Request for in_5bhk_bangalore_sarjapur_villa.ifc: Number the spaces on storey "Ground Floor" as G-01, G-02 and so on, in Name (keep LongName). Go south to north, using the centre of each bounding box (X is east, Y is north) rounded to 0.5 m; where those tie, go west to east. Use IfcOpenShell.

First a look at what the model holds.

```python
import ifcopenshell
import ifcopenshell.util.element
import ifcopenshell.util.placement

model = ifcopenshell.open("in_5bhk_bangalore_sarjapur_villa.ifc")
print(model.schema)
storey = next(s for s in model.by_type("IfcBuildingStorey") if s.Name == "Ground Floor")
spaces = [e for e in ifcopenshell.util.element.get_decomposition(storey) if e.is_a("IfcSpace")]
for e in sorted(spaces, key=lambda e: e.id()):
    origin = ifcopenshell.util.placement.get_local_placement(e.ObjectPlacement)[:3, 3]
    print(e.id(), e.Name, e.LongName, origin.round(2) + 0.0, sep=" | ")
```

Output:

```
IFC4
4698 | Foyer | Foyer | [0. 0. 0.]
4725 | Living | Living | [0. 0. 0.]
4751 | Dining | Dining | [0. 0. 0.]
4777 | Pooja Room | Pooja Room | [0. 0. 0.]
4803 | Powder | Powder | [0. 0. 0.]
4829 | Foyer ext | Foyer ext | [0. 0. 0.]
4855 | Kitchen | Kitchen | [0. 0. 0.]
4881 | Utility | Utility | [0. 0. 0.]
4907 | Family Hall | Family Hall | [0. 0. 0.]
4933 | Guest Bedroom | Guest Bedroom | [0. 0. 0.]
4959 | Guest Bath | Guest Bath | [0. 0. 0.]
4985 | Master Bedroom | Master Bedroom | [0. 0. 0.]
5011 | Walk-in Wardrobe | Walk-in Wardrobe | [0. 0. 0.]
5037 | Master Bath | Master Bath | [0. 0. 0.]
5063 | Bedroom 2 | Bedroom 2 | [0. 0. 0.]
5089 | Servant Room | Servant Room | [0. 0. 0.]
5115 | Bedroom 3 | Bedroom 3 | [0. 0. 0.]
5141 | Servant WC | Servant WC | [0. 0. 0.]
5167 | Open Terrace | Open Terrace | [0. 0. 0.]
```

```python
import ifcopenshell
import ifcopenshell.geom
import ifcopenshell.util.element
import ifcopenshell.util.shape

model = ifcopenshell.open("in_5bhk_bangalore_sarjapur_villa.ifc")
settings = ifcopenshell.geom.settings()
settings.set("use-world-coords", True)


def centre(element):
    shape = ifcopenshell.geom.create_shape(settings, element)
    return ifcopenshell.util.shape.get_bbox_centroid(shape.geometry)


storey = next(s for s in model.by_type("IfcBuildingStorey") if s.Name == "Ground Floor")
spaces = [e for e in ifcopenshell.util.element.get_decomposition(storey) if e.is_a("IfcSpace")]

# Insertion points can sit at a corner or the storey origin, so sort by the geometry (in metres).
centres = {e: centre(e) for e in spaces}
spaces.sort(key=lambda e: (round(centres[e][1] / 0.5), centres[e][0]))

for i, e in enumerate(spaces, start=1):
    number = f"G-{i:02d}"
    e.Name = number
    print(e.id(), number)

model.write("in_5bhk_bangalore_sarjapur_villa-out.ifc")
```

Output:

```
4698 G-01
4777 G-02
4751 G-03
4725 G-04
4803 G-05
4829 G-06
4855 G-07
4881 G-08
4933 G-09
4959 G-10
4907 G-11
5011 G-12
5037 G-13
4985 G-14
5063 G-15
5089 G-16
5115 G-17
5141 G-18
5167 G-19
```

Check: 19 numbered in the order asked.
